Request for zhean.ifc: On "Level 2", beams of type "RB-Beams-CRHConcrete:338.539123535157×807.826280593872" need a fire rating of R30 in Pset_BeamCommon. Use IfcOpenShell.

First a look at what the model holds.

```python
import ifcopenshell
import ifcopenshell.util.element

model = ifcopenshell.open("zhean.ifc")
print(model.schema)
storey = next(s for s in model.by_type("IfcBuildingStorey") if s.Name == "Level 2")
beams = [e for e in ifcopenshell.util.element.get_decomposition(storey) if e.is_a("IfcBeam")]
seen = {}
for e in beams:
    element_type = ifcopenshell.util.element.get_type(e)
    key = (element_type.Name if element_type != e and element_type else None, ifcopenshell.util.element.get_pset(e, "Pset_BeamCommon", "FireRating"))
    seen[key] = seen.get(key, 0) + 1
for (name, value), count in sorted(seen.items(), key=str):
    print(count, "x", name, "|", value)
```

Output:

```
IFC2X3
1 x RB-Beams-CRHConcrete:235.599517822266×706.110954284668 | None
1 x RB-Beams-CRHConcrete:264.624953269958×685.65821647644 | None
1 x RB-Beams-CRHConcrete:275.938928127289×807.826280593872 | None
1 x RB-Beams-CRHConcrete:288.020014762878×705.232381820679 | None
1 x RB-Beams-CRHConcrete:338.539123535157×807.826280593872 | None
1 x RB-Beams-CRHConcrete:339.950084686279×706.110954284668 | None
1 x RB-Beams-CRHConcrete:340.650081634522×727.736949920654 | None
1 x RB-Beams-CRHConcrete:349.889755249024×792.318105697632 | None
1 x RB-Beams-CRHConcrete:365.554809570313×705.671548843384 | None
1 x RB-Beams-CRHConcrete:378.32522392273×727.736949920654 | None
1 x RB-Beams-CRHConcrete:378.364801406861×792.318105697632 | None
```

```python
import ifcopenshell
import ifcopenshell.api.pset
import ifcopenshell.util.element

model = ifcopenshell.open("zhean.ifc")

storey = next(s for s in model.by_type("IfcBuildingStorey") if s.Name == "Level 2")
beams = [e for e in ifcopenshell.util.element.get_decomposition(storey) if e.is_a("IfcBeam")]

count = 0
for e in beams:
    element_type = ifcopenshell.util.element.get_type(e)
    if element_type in (None, e) or element_type.Name != "RB-Beams-CRHConcrete:338.539123535157×807.826280593872":
        continue
    # add_pset returns the element's existing set when there is one.
    pset = ifcopenshell.api.pset.add_pset(model, product=e, name="Pset_BeamCommon")
    ifcopenshell.api.pset.edit_pset(model, pset=pset, properties={"FireRating": "R30"})
    count += 1

print(count, "beams updated")

model.write("zhean_rev.ifc")
```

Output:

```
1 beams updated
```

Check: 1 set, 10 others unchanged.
